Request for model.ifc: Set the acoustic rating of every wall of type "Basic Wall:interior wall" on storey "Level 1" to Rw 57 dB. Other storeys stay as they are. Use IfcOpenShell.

First a look at what the model holds.

```python
import ifcopenshell
import ifcopenshell.util.element

model = ifcopenshell.open("model.ifc")
print(model.schema)
storey = next(s for s in model.by_type("IfcBuildingStorey") if s.Name == "Level 1")
walls = [e for e in ifcopenshell.util.element.get_decomposition(storey) if e.is_a("IfcWall")]
seen = {}
for e in walls:
    element_type = ifcopenshell.util.element.get_type(e)
    key = (element_type.Name if element_type != e and element_type else None, ifcopenshell.util.element.get_pset(e, "Pset_WallCommon", "AcousticRating"))
    seen[key] = seen.get(key, 0) + 1
for (name, value), count in sorted(seen.items(), key=str):
    print(count, "x", name, "|", value)
```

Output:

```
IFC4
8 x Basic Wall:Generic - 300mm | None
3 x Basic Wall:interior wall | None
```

```python
import ifcopenshell
import ifcopenshell.api.pset
import ifcopenshell.util.element

model = ifcopenshell.open("model.ifc")

storey = next(s for s in model.by_type("IfcBuildingStorey") if s.Name == "Level 1")
walls = [e for e in ifcopenshell.util.element.get_decomposition(storey) if e.is_a("IfcWall")]

count = 0
for e in walls:
    element_type = ifcopenshell.util.element.get_type(e)
    if element_type in (None, e) or element_type.Name != "Basic Wall:interior wall":
        continue
    # add_pset returns the element's existing set when there is one.
    pset = ifcopenshell.api.pset.add_pset(model, product=e, name="Pset_WallCommon")
    ifcopenshell.api.pset.edit_pset(model, pset=pset, properties={"AcousticRating": "Rw 57 dB"})
    count += 1

print(count, "walls updated")

model.write("model-out.ifc")
```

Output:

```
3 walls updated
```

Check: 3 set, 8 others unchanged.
